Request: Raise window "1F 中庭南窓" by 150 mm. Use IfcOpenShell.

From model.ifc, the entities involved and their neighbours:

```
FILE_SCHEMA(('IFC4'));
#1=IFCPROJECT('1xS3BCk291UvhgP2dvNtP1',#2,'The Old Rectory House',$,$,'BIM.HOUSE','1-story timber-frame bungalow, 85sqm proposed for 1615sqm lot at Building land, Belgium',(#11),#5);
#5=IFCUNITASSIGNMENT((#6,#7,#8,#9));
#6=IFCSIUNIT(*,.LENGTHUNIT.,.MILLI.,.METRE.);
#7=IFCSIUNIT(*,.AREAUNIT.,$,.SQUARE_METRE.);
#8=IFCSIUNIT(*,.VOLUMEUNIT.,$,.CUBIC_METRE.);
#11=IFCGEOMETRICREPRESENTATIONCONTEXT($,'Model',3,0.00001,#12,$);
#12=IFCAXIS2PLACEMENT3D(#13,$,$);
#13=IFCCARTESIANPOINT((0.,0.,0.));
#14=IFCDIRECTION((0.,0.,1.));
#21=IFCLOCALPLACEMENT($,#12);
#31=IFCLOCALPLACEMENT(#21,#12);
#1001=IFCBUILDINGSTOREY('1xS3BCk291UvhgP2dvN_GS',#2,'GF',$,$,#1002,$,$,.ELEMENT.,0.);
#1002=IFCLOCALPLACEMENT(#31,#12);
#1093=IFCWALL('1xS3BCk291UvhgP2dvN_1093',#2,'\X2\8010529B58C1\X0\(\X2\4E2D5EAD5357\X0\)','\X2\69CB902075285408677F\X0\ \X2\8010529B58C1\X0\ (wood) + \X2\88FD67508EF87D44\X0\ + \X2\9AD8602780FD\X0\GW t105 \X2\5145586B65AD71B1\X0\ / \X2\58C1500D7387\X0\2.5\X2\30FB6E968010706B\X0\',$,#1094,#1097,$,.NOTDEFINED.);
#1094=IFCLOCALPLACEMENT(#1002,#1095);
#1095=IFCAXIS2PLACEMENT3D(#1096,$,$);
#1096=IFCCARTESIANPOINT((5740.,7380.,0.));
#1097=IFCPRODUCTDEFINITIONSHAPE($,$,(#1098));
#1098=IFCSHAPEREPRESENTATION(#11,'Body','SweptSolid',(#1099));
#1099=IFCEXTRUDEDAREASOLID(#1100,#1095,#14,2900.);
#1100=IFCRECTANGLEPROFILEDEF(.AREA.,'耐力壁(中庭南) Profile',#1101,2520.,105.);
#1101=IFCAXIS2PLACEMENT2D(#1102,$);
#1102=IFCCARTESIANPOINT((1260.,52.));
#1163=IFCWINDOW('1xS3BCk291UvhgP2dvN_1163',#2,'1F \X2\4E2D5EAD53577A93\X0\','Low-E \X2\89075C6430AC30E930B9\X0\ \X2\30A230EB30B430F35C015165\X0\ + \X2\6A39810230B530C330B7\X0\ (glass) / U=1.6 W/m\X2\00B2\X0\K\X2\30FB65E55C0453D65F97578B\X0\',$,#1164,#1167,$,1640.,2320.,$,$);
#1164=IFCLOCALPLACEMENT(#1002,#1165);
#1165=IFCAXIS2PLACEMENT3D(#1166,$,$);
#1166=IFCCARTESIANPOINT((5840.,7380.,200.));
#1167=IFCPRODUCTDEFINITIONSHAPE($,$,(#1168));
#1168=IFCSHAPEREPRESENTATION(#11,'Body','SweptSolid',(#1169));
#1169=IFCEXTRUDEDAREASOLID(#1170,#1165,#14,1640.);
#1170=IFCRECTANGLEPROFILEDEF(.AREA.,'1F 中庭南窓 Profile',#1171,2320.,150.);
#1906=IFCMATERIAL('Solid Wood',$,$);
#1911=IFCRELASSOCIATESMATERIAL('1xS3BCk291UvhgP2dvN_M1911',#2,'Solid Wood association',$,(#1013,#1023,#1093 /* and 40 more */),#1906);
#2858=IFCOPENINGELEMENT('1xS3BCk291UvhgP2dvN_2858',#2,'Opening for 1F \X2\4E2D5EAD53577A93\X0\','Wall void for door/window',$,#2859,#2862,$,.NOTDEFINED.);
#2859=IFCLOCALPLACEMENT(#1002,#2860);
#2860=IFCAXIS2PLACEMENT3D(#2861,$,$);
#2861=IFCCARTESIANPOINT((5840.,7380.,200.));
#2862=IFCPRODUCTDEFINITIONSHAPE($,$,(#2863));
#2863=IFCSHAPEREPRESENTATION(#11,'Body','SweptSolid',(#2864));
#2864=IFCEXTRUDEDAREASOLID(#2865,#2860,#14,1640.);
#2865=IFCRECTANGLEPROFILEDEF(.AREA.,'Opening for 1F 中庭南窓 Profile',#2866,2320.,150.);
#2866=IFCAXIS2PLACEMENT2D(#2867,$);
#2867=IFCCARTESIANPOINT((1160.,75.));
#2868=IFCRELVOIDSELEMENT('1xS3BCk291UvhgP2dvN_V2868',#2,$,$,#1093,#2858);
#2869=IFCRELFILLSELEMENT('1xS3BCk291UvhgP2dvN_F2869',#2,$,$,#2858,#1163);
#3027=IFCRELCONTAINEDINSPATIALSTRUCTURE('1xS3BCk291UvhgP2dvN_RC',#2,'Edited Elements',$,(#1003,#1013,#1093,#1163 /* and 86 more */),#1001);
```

```python
import numpy as np
import ifcopenshell
import ifcopenshell.api.geometry
import ifcopenshell.util.placement
import ifcopenshell.util.unit

model = ifcopenshell.open("model.ifc")
unit_scale = ifcopenshell.util.unit.calculate_unit_scale(model)

window = model.by_guid("1xS3BCk291UvhgP2dvN_1163")
opening = window.FillsVoids[0].RelatingOpeningElement
dz = 150.0

shift = np.array([0.0, 0.0, dz])
# The window is not placed relative to its opening, so move both.
for product in (opening, window):
    matrix = ifcopenshell.util.placement.get_local_placement(product.ObjectPlacement)
    matrix[:3, 3] += shift
    ifcopenshell.api.geometry.edit_object_placement(model, product=product, matrix=matrix, is_si=False)

print(f"moved by {dz * unit_scale:+.3f} m")

model.write("model-out.ifc")
```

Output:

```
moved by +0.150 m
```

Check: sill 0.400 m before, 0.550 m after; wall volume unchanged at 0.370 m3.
